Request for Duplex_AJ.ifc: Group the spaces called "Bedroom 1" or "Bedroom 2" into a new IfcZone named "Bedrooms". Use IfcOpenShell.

First a look at what the model holds.

```python
import ifcopenshell

model = ifcopenshell.open("Duplex_AJ.ifc")
print(model.schema)
seen = {}
for space in model.by_type("IfcSpace"):
    seen[space.LongName] = seen.get(space.LongName, 0) + 1
for name, count in sorted(seen.items(), key=str):
    print(count, "x", name)
print("zones:", [z.Name for z in model.by_type("IfcZone")][:20])
```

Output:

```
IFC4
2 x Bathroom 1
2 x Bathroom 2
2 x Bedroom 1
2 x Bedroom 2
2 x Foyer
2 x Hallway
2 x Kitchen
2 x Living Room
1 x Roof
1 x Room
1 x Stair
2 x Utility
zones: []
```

```python
import ifcopenshell
import ifcopenshell.api.group
import ifcopenshell.api.root

model = ifcopenshell.open("Duplex_AJ.ifc")

names = {"Bedroom 1", "Bedroom 2"}
spaces = [s for s in model.by_type("IfcSpace") if s.LongName in names]

zone = ifcopenshell.api.root.create_entity(model, ifc_class="IfcZone", name="Bedrooms")
ifcopenshell.api.group.assign_group(model, products=spaces, group=zone)
print(len(spaces), "spaces in", zone.Name)

model.write("Duplex_AJ_edited.ifc")
```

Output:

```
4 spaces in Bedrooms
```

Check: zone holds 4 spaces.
